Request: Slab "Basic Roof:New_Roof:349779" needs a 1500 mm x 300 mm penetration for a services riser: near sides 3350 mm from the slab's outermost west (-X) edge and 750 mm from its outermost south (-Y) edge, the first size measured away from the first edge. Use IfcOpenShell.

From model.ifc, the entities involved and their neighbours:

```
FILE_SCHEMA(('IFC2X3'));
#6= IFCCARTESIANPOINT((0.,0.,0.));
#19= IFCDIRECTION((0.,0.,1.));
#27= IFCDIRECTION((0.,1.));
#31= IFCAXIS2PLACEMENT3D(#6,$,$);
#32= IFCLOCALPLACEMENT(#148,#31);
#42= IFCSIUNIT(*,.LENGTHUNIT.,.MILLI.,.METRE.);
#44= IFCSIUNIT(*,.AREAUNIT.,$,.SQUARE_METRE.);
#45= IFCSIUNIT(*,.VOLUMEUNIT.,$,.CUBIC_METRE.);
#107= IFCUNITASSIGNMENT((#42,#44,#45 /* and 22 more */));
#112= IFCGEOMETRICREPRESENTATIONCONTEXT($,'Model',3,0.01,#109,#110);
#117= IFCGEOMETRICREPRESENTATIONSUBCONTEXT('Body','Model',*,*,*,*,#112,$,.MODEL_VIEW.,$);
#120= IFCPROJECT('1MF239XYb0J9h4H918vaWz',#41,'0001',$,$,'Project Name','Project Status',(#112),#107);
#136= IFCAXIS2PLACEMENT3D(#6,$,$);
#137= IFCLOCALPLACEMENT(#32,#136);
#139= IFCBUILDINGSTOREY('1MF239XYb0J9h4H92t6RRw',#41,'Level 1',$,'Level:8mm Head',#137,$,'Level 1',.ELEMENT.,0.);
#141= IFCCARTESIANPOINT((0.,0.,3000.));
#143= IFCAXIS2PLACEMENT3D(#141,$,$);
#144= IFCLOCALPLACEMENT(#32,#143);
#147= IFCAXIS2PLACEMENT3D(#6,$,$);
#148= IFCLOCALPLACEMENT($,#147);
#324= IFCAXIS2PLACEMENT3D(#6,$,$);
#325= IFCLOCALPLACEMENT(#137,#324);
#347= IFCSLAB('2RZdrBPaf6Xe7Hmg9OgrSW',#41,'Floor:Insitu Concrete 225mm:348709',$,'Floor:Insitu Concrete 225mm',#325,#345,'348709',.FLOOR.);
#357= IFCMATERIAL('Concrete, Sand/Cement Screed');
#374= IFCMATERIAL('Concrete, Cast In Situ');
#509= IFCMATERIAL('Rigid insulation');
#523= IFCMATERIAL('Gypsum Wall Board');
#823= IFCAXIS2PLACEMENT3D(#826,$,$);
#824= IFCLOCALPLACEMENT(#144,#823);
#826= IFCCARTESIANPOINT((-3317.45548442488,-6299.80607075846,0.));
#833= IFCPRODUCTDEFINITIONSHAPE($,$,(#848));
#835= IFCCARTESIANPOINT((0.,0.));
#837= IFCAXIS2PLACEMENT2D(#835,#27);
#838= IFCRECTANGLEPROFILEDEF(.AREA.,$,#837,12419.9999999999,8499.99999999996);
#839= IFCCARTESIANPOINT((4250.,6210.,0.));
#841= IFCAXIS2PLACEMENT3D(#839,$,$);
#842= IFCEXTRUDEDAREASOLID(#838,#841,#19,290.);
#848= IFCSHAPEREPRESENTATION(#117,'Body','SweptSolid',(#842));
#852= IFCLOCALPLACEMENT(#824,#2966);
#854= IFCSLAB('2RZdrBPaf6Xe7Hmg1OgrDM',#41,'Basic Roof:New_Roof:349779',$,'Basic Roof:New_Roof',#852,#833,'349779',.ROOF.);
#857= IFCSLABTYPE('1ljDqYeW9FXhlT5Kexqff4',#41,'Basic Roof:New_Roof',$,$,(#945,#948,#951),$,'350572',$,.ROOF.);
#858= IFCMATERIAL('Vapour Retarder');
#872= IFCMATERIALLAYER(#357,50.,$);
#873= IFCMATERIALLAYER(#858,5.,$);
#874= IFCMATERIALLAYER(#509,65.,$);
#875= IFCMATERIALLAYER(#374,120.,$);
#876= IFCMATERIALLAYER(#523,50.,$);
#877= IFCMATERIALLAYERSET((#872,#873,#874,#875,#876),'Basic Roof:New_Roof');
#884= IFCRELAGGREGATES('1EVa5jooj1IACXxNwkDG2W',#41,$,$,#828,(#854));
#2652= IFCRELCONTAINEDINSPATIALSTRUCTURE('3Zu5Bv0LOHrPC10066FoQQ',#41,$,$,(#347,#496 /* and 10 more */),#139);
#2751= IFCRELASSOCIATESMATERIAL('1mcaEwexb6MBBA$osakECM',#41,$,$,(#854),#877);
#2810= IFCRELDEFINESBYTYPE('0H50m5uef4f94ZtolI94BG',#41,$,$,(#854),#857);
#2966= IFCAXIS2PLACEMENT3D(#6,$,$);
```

```python
import numpy as np
import ifcopenshell
import ifcopenshell.api.feature
import ifcopenshell.api.geometry
import ifcopenshell.api.root
import ifcopenshell.geom
import ifcopenshell.util.placement
import ifcopenshell.util.representation
import ifcopenshell.util.shape
import ifcopenshell.util.unit

model = ifcopenshell.open("model.ifc")
unit_scale = ifcopenshell.util.unit.calculate_unit_scale(model)
settings = ifcopenshell.geom.settings()


def volume(element):
    """Net volume in cubic metres, openings subtracted."""
    shape = ifcopenshell.geom.create_shape(settings, element)
    return ifcopenshell.util.shape.get_volume(shape.geometry)


slab = model.by_guid("2RZdrBPaf6Xe7Hmg1OgrDM")
before = volume(slab)

# Extent in the slab's own axes, in metres. The edges named are its -X and -Y sides.
slab_shape = ifcopenshell.geom.create_shape(settings, slab)
vertices = ifcopenshell.util.shape.get_vertices(slab_shape.geometry)
x_min, y_min, bottom = vertices.min(axis=0)
top = vertices[:, 2].max()

opening = ifcopenshell.api.root.create_entity(model, ifc_class="IfcOpeningElement", name="Services riser opening")
context = ifcopenshell.util.representation.get_context(model, "Model", "Body", "MODEL_VIEW")
width, depth = 1.5, 0.3
outline = [(0.0, 0.0), (width, 0.0), (width, depth), (0.0, depth), (0.0, 0.0)]
# Overshoot both faces by 50 mm so the cut is clean.
shape = ifcopenshell.api.geometry.add_slab_representation(
    model, context=context, depth=top - bottom + 0.1, polyline=outline
)
ifcopenshell.api.geometry.assign_representation(model, product=opening, representation=shape)

matrix = ifcopenshell.util.placement.get_local_placement(slab.ObjectPlacement)
matrix[:, 3] = matrix @ np.append(np.array([x_min + 3.35, y_min + 0.75, bottom - 0.05]) / unit_scale, 1.0)
ifcopenshell.api.geometry.edit_object_placement(model, product=opening, matrix=matrix, is_si=False)
ifcopenshell.api.feature.add_feature(model, feature=opening, element=slab)

after = volume(slab)

print(f"slab volume {before:.3f} -> {after:.3f} m3")

model.write("model_updated.ifc")
```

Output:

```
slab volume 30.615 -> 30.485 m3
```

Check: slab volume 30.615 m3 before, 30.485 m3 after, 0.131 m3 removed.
